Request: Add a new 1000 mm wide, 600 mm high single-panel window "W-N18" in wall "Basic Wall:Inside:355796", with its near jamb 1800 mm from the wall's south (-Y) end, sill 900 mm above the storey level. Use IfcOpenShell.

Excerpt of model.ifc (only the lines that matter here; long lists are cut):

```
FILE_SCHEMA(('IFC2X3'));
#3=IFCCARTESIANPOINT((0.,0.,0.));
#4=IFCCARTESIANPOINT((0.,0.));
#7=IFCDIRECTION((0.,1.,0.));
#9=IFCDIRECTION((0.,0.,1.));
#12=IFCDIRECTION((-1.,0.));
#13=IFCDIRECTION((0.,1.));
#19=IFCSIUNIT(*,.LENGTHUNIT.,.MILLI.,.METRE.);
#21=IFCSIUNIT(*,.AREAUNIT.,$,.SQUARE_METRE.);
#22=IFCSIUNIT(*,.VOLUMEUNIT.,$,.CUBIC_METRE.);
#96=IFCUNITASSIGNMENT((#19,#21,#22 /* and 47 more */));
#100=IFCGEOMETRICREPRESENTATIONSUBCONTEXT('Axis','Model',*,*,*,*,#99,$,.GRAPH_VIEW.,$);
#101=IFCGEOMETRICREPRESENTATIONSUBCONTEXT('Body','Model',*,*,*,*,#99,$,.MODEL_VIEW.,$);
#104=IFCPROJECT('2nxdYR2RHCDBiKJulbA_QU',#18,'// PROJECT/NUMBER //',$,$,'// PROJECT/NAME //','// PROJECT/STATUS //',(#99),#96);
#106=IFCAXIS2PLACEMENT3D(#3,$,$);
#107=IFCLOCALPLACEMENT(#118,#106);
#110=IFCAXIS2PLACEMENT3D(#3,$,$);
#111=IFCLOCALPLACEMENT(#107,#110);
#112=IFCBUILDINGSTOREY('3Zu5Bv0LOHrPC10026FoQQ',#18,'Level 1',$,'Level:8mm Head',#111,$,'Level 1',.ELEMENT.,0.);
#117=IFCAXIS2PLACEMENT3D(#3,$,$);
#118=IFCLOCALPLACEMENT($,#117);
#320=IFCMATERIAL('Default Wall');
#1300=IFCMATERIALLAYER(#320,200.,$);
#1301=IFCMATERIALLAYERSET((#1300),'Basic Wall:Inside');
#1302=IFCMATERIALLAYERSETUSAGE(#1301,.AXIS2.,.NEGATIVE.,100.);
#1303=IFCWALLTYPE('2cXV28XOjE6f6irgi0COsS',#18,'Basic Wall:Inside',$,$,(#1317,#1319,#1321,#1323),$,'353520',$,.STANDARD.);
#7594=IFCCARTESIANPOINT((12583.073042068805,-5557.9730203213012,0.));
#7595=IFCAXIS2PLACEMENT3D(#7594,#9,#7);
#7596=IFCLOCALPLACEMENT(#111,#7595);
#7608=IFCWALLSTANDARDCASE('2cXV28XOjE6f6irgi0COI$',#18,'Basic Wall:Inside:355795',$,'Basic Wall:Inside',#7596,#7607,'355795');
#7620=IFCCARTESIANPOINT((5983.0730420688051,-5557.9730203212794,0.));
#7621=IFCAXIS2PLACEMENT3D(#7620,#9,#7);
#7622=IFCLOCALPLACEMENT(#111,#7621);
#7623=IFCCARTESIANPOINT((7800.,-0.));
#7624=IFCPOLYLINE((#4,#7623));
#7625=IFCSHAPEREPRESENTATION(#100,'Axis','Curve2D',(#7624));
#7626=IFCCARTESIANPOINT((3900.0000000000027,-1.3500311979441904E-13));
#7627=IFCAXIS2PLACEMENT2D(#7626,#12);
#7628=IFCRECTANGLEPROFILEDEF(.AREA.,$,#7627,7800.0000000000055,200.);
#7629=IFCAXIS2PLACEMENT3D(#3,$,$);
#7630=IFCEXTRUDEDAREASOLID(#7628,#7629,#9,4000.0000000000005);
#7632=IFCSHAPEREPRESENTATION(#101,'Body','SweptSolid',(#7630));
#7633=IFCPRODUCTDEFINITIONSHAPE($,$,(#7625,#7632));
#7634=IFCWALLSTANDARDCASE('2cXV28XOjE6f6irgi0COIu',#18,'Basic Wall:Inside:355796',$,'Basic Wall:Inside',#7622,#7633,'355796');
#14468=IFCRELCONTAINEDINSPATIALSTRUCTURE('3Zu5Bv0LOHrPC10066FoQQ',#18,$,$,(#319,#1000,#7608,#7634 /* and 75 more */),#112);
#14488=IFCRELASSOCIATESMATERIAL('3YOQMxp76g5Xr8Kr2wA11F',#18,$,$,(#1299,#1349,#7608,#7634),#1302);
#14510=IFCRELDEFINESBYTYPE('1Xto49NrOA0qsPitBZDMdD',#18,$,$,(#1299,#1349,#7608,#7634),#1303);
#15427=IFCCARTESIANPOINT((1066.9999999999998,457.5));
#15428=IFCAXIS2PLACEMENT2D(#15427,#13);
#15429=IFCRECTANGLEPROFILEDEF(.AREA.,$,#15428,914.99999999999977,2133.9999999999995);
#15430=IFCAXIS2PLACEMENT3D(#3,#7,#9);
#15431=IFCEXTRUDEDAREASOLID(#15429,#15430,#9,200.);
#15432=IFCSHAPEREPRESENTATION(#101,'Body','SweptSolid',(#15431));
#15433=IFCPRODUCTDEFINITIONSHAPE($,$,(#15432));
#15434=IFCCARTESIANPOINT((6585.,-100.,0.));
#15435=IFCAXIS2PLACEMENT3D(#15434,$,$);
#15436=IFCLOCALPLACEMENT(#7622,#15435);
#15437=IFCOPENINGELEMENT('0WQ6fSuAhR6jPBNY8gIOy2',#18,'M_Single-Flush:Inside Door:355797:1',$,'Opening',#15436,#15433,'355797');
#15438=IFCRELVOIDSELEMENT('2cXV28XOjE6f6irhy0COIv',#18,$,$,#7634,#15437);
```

```python
import numpy as np
import ifcopenshell
import ifcopenshell.api.feature
import ifcopenshell.api.geometry
import ifcopenshell.api.root
import ifcopenshell.api.spatial
import ifcopenshell.api.type
import ifcopenshell.geom
import ifcopenshell.util.element
import ifcopenshell.util.placement
import ifcopenshell.util.representation
import ifcopenshell.util.shape
import ifcopenshell.util.unit

model = ifcopenshell.open("model.ifc")
unit_scale = ifcopenshell.util.unit.calculate_unit_scale(model)
settings = ifcopenshell.geom.settings()


def volume(element):
    """Net volume in cubic metres, openings subtracted."""
    shape = ifcopenshell.geom.create_shape(settings, element)
    return ifcopenshell.util.shape.get_volume(shape.geometry)


wall = model.by_id(7634)
storey = ifcopenshell.util.element.get_container(wall, ifc_class="IfcBuildingStorey")
context = ifcopenshell.util.representation.get_context(model, "Model", "Body", "MODEL_VIEW")
before = volume(wall)

width, height, from_end, sill = 1, 0.6, 1.8, 0.9  # metres

# The wall runs along its own X axis, and the end named is its -X end.
wall_shape = ifcopenshell.geom.create_shape(settings, wall)
x, y, z = ifcopenshell.util.shape.get_vertices(wall_shape.geometry).T
start = x.min() + from_end
face, thickness = float(y.min()), float(y.max() - y.min())
wall_matrix = ifcopenshell.util.placement.get_local_placement(wall.ObjectPlacement)
level = ifcopenshell.util.placement.get_local_placement(storey.ObjectPlacement)[2, 3]


def in_wall(x, y):
    """Placement at x, y metres in the wall's axes, at sill height."""
    matrix = wall_matrix.copy()
    matrix[:, 3] = wall_matrix @ np.array([x / unit_scale, y / unit_scale, 0.0, 1.0])
    matrix[2, 3] = level + sill / unit_scale
    return matrix


# Opening: a box that overshoots both wall faces by 50 mm.
opening = ifcopenshell.api.root.create_entity(model, ifc_class="IfcOpeningElement")
box = ifcopenshell.api.geometry.add_wall_representation(
    model, context=context, length=width, height=height, thickness=thickness + 0.1
)
ifcopenshell.api.geometry.assign_representation(model, product=opening, representation=box)
ifcopenshell.api.geometry.edit_object_placement(model, product=opening, matrix=in_wall(start, face - 0.05), is_si=False)
ifcopenshell.api.feature.add_feature(model, feature=opening, element=wall)

window = ifcopenshell.api.root.create_entity(model, ifc_class="IfcWindow", name="W-N18")
window.OverallWidth, window.OverallHeight = width / unit_scale, height / unit_scale
body = ifcopenshell.api.geometry.add_window_representation(
    model,
    context=context,
    overall_width=window.OverallWidth,
    overall_height=window.OverallHeight,
    partition_type="SINGLE_PANEL",
)
ifcopenshell.api.geometry.assign_representation(model, product=window, representation=body)
ifcopenshell.api.spatial.assign_container(model, products=[window], relating_structure=storey)
fills = ifcopenshell.api.feature.add_filling(model, opening=opening, element=window)
fills.OwnerHistory = window.OwnerHistory  # required in IFC2X3

# IFC2X3 keeps the operation on the window style.
style = ifcopenshell.api.root.create_entity(model, ifc_class="IfcWindowStyle", name="W-N18")
style.OperationType, style.ConstructionType = "SINGLE_PANEL", "NOTDEFINED"
style.ParameterTakesPrecedence = style.Sizeable = False
ifcopenshell.api.type.assign_type(model, related_objects=[window], relating_type=style)

# Centre the window in the wall's thickness.
ifcopenshell.api.geometry.edit_object_placement(model, product=window, matrix=in_wall(start, face), is_si=False)
window_shape = ifcopenshell.geom.create_shape(settings, window)
depth = ifcopenshell.util.shape.get_vertices(window_shape.geometry)[:, 1]
offset = face + thickness / 2 - (depth.min() + depth.max()) / 2
ifcopenshell.api.geometry.edit_object_placement(model, product=window, matrix=in_wall(start, offset), is_si=False)

after = volume(wall)

print(f"wall volume {before:.3f} -> {after:.3f} m3")

model.write("model-out.ifc")
```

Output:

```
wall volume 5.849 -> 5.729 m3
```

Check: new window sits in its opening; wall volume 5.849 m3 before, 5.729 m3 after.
